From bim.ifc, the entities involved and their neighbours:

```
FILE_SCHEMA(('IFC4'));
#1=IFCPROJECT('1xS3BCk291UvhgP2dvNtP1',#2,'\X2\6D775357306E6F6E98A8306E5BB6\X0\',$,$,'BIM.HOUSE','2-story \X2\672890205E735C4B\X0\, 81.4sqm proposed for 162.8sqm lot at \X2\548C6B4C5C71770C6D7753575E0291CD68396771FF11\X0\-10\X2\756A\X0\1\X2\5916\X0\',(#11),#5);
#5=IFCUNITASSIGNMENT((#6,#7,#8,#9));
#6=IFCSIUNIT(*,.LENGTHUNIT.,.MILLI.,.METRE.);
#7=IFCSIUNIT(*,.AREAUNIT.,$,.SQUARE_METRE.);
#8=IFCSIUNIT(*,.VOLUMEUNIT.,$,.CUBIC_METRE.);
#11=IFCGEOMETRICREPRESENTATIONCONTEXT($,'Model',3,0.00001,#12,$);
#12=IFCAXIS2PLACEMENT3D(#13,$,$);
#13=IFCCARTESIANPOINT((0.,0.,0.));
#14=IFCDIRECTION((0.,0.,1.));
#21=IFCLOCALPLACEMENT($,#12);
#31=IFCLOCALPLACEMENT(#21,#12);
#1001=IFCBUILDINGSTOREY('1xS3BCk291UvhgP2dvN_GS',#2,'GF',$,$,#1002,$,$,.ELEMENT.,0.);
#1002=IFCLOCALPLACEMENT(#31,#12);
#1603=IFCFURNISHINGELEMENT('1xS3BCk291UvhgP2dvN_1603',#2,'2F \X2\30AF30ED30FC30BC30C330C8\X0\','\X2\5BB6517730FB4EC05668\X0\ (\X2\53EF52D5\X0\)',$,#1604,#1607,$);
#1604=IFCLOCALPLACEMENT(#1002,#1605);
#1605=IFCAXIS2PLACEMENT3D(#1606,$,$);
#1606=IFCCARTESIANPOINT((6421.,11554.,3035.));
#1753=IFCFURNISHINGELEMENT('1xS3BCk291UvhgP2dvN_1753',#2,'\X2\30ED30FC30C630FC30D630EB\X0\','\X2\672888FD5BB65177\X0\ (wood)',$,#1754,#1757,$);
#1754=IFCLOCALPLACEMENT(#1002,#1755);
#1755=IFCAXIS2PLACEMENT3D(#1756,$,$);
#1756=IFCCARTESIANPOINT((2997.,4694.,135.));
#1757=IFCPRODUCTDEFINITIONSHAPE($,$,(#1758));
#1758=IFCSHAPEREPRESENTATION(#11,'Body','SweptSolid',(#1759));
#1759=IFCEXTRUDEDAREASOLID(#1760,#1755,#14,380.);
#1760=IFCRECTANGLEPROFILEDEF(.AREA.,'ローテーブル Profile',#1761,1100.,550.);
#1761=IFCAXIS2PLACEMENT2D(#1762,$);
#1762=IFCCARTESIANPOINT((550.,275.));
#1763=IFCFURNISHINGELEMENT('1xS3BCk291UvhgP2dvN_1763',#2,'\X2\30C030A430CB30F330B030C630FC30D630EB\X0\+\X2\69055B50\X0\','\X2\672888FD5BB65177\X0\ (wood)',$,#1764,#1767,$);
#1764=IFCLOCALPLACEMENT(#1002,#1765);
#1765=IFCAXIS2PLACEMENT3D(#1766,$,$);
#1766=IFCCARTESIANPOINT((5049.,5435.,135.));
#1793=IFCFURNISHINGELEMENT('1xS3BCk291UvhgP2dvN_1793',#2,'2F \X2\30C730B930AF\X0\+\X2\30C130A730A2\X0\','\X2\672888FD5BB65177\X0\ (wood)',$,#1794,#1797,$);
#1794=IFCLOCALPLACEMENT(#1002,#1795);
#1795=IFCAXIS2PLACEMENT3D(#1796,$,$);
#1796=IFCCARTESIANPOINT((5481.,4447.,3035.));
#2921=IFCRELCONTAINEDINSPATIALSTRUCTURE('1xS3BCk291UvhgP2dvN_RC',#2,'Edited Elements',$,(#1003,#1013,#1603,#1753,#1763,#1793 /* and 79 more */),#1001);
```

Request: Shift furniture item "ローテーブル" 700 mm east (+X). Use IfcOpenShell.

```python
import ifcopenshell
import ifcopenshell.api.geometry
import ifcopenshell.util.placement

model = ifcopenshell.open("bim.ifc")

item = model.by_guid("1xS3BCk291UvhgP2dvN_1753")
matrix = ifcopenshell.util.placement.get_local_placement(item.ObjectPlacement)
matrix[0, 3] += 700.0
ifcopenshell.api.geometry.edit_object_placement(model, product=item, matrix=matrix, is_si=False)

print(ifcopenshell.util.placement.get_local_placement(item.ObjectPlacement).round(3) + 0.0)

model.write("bim_edited.ifc")
```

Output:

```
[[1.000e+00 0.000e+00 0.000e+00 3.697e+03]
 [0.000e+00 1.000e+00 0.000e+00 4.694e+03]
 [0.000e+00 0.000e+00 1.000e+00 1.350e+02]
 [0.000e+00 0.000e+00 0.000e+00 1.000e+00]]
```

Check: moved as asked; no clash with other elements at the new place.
